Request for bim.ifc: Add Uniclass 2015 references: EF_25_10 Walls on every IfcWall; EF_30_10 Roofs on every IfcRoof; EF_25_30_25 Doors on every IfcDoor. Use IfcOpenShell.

First a look at what the model holds.

```python
import ifcopenshell

model = ifcopenshell.open("bim.ifc")
print(model.schema)
print("classifications:", [c.Name for c in model.by_type("IfcClassification")])
for ifc_class in ("IfcDoor", "IfcRoof", "IfcStair", "IfcWall", "IfcWindow"):
    print(ifc_class, len(model.by_type(ifc_class)))
```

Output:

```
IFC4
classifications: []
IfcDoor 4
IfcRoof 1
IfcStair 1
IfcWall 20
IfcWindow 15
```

```python
import ifcopenshell
import ifcopenshell.api.classification

model = ifcopenshell.open("bim.ifc")

system = ifcopenshell.api.classification.add_classification(model, classification="Uniclass 2015")

codes = {
    "IfcWall": ("EF_25_10", "Walls"),
    "IfcRoof": ("EF_30_10", "Roofs"),
    "IfcDoor": ("EF_25_30_25", "Doors"),
}
for ifc_class, (code, name) in codes.items():
    products = model.by_type(ifc_class)
    ifcopenshell.api.classification.add_reference(
        model, products=products, classification=system, identification=code, name=name
    )
    print(code, len(products))

model.write("bim_updated.ifc")
```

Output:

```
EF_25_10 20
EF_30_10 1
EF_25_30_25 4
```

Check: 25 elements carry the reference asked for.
